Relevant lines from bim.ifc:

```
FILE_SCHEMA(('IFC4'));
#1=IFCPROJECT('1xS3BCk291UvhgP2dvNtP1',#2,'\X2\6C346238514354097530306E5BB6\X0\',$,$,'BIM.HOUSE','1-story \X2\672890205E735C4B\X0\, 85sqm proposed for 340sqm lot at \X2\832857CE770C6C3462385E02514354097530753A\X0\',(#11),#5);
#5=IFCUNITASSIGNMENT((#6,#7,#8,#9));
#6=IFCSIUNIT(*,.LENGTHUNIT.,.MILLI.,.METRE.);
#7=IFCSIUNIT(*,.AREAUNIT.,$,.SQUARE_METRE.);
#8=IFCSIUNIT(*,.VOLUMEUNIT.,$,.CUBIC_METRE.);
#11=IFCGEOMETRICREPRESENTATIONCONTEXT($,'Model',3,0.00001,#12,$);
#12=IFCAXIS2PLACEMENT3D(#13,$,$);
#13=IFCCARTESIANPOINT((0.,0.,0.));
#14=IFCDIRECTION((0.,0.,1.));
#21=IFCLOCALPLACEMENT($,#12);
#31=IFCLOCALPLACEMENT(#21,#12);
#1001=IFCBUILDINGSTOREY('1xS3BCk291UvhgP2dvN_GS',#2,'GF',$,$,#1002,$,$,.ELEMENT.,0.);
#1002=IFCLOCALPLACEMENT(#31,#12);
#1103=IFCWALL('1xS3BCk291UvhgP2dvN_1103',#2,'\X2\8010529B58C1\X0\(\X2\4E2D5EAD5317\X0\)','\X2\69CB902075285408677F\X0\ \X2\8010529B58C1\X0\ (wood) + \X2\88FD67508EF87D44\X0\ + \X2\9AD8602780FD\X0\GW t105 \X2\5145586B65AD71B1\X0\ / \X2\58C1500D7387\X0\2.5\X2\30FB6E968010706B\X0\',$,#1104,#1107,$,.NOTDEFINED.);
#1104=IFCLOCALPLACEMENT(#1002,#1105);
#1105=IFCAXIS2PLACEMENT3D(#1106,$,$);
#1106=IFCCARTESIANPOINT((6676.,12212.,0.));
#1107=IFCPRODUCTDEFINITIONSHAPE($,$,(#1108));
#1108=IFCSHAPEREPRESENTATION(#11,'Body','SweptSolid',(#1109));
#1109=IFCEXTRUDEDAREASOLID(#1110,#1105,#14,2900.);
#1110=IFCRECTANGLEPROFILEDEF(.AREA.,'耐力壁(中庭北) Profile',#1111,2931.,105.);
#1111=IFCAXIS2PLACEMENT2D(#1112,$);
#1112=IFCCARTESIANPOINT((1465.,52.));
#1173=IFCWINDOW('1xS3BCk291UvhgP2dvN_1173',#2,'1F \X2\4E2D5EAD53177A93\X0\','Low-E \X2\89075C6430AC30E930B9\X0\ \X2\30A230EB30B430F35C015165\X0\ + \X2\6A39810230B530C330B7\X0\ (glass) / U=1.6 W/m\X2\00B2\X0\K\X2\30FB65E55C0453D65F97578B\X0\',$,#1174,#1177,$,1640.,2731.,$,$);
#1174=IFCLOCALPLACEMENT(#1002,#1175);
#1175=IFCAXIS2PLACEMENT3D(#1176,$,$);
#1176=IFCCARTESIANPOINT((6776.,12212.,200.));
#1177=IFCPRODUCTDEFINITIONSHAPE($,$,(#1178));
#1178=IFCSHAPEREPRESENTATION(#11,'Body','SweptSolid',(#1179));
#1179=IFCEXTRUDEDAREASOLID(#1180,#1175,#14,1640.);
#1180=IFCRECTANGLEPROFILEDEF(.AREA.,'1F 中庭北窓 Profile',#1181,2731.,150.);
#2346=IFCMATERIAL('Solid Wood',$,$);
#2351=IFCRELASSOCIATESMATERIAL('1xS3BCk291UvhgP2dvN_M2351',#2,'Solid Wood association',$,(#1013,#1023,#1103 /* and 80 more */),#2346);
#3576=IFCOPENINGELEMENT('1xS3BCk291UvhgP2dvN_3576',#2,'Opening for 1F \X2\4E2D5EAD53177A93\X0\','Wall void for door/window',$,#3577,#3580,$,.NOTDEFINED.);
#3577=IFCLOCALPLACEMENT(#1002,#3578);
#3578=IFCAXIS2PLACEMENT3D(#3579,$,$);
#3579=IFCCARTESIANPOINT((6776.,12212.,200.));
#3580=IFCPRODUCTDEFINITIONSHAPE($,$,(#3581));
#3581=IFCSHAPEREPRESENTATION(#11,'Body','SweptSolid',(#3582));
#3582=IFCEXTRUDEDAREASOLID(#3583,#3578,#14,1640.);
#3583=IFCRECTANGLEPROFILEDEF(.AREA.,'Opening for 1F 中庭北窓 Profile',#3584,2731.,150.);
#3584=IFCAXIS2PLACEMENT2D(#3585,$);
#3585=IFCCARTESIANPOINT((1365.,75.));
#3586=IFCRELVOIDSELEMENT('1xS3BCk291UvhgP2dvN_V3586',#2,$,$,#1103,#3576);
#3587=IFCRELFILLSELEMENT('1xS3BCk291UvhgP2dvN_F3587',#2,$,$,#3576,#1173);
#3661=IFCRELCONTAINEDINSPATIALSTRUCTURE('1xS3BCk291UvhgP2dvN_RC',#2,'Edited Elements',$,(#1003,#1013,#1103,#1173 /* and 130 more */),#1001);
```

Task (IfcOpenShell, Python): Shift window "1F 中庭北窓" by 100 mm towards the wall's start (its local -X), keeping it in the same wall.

```python
import ifcopenshell
import ifcopenshell.api.geometry
import ifcopenshell.util.placement
import ifcopenshell.util.unit

model = ifcopenshell.open("bim.ifc")
unit_scale = ifcopenshell.util.unit.calculate_unit_scale(model)

window = model.by_guid("1xS3BCk291UvhgP2dvN_1173")
opening = window.FillsVoids[0].RelatingOpeningElement
wall = opening.VoidsElements[0].RelatingBuildingElement

wall_matrix = ifcopenshell.util.placement.get_local_placement(wall.ObjectPlacement)
shift = wall_matrix[:3, 0] * -0.1 / unit_scale
before = ifcopenshell.util.placement.get_local_placement(window.ObjectPlacement)[:3, 3].copy()

# The window is not placed relative to its opening, so move both.
for product in (opening, window):
    matrix = ifcopenshell.util.placement.get_local_placement(product.ObjectPlacement)
    matrix[:3, 3] += shift
    ifcopenshell.api.geometry.edit_object_placement(model, product=product, matrix=matrix, is_si=False)

after = ifcopenshell.util.placement.get_local_placement(window.ObjectPlacement)[:3, 3]
print("window moved by", (after - before).round(3) + 0.0)

model.write("bim_v2.ifc")
```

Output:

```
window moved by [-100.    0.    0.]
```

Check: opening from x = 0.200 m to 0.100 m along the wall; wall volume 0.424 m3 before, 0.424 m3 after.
